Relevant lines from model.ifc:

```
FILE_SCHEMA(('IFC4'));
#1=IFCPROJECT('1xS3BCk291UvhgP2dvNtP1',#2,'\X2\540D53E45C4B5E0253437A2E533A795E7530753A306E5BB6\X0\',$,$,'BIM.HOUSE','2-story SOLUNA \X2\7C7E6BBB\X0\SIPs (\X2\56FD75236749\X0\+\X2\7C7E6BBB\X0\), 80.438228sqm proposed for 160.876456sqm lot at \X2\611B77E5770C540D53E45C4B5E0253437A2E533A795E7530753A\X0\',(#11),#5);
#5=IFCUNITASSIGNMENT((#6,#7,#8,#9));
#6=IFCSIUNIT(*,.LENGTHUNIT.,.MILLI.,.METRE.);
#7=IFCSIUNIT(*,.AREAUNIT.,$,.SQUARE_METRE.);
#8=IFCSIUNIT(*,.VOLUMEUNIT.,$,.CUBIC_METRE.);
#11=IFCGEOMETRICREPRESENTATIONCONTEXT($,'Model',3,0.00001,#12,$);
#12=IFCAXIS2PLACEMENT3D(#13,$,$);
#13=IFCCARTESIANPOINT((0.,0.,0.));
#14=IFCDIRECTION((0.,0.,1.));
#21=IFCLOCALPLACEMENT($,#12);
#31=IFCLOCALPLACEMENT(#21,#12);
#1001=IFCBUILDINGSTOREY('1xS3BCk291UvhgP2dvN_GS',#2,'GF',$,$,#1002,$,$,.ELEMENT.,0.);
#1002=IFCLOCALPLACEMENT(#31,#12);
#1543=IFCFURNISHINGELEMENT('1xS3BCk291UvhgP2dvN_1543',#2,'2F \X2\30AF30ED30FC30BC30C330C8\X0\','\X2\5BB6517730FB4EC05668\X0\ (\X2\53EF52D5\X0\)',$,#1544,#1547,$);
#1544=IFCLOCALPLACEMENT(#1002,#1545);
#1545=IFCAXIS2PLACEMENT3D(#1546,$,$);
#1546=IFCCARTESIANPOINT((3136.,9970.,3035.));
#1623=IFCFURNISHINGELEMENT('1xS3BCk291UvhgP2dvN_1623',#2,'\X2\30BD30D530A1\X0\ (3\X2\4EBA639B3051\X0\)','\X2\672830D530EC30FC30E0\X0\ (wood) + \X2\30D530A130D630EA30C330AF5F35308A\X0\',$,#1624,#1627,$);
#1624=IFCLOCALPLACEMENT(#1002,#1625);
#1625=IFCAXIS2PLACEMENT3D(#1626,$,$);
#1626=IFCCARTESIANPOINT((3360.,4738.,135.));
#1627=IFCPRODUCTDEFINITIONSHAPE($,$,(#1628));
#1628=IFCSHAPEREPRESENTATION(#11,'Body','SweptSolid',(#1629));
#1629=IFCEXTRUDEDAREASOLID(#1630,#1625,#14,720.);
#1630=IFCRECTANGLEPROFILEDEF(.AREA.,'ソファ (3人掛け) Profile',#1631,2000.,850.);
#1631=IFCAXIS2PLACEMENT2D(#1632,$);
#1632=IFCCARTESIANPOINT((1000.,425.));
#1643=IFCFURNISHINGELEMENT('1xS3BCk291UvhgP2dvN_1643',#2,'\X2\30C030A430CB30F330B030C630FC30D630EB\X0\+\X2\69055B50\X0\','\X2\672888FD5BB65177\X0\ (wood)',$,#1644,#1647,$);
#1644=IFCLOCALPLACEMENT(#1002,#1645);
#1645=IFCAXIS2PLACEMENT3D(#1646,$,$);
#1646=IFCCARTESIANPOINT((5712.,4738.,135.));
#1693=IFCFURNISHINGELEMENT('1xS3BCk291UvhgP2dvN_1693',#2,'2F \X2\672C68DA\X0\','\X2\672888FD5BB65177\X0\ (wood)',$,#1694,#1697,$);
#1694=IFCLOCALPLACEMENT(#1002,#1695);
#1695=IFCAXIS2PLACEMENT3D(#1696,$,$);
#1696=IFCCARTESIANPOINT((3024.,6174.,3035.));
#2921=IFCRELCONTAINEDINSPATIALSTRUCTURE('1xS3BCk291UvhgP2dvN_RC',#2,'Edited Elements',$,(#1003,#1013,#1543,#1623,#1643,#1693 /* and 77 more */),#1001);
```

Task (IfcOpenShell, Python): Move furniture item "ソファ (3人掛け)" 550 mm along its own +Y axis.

```python
import ifcopenshell
import ifcopenshell.api.geometry
import ifcopenshell.util.placement
import ifcopenshell.util.unit

model = ifcopenshell.open("model.ifc")
unit_scale = ifcopenshell.util.unit.calculate_unit_scale(model)

item = model.by_id(1623)
matrix = ifcopenshell.util.placement.get_local_placement(item.ObjectPlacement)
matrix[:3, 3] += matrix[:3, 1] * 0.55 / unit_scale
ifcopenshell.api.geometry.edit_object_placement(model, product=item, matrix=matrix, is_si=False)

print(ifcopenshell.util.placement.get_local_placement(item.ObjectPlacement).round(3) + 0.0)

model.write("model_rev.ifc")
```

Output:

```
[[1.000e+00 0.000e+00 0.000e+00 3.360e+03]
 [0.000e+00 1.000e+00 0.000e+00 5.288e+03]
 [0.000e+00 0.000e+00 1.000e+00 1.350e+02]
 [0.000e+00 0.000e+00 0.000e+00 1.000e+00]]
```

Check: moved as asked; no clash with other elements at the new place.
